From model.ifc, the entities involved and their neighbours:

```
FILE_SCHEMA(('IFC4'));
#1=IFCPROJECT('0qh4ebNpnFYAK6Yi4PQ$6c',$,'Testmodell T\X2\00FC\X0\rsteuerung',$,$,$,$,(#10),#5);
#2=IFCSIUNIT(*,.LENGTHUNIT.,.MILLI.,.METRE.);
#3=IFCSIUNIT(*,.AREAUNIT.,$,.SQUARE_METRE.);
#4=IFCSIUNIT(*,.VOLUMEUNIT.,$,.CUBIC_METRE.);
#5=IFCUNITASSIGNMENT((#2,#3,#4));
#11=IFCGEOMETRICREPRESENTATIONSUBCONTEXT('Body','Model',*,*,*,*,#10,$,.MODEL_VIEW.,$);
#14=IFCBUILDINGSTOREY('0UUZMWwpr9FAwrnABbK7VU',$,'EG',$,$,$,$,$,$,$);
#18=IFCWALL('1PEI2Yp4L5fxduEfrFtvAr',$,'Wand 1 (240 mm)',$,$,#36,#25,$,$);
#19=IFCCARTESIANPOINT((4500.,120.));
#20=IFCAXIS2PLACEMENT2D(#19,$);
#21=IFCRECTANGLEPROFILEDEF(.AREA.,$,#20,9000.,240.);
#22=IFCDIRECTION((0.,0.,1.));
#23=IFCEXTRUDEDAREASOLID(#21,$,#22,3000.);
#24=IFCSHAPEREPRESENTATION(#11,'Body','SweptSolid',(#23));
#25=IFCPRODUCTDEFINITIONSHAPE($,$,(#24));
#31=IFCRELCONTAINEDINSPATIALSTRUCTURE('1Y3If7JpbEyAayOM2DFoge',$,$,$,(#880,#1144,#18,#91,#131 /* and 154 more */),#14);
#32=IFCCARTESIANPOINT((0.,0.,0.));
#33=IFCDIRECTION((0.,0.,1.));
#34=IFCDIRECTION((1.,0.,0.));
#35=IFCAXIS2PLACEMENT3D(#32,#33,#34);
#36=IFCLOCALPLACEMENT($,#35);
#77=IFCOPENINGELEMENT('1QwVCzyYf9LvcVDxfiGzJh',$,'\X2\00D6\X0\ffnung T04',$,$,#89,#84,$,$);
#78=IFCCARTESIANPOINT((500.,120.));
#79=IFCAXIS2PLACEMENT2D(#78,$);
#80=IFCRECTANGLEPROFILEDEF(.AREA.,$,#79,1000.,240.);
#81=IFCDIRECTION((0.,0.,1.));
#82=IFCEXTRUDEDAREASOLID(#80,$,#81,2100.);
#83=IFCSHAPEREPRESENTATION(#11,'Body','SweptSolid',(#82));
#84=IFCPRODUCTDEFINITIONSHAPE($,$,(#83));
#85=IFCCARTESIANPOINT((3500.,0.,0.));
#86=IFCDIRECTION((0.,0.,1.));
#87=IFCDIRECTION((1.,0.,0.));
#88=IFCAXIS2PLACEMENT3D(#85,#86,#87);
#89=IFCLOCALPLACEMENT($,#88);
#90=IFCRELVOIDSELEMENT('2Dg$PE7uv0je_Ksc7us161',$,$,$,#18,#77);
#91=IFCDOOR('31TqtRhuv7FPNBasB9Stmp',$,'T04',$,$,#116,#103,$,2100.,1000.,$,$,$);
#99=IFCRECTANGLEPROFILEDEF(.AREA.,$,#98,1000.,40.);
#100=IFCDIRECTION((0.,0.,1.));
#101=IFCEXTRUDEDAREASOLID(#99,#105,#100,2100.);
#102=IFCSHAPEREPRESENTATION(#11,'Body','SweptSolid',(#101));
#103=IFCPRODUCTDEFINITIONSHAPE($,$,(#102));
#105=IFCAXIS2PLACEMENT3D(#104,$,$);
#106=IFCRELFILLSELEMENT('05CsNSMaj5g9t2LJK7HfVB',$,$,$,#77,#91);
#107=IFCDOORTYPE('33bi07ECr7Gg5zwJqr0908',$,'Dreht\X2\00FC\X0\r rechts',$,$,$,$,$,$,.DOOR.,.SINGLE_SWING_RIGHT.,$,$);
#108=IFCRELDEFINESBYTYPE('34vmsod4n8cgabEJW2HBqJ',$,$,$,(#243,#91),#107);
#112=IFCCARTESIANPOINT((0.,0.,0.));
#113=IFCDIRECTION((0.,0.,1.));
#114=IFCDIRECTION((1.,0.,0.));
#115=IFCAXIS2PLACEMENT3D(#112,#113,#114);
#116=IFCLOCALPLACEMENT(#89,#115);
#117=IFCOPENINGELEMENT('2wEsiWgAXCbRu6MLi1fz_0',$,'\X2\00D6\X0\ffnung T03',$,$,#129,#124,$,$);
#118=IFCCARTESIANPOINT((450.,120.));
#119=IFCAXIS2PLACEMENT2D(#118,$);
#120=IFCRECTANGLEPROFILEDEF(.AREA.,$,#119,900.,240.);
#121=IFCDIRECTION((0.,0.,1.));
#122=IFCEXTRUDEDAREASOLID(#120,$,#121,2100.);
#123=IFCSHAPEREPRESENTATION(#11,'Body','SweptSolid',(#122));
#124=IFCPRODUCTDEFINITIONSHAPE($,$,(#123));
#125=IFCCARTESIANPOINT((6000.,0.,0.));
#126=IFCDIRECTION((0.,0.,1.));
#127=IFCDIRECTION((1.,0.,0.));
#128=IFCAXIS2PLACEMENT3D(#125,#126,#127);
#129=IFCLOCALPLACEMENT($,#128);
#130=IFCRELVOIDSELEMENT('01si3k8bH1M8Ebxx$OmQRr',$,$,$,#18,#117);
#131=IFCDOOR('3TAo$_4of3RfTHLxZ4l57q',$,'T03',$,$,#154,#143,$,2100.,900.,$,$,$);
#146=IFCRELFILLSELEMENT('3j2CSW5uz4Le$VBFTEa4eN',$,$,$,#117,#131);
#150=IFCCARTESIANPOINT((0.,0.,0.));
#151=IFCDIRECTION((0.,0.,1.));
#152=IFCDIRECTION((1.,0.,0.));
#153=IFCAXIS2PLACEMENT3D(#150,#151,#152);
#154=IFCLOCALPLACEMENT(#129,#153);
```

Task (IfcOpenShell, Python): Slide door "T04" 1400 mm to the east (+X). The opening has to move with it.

```python
import ifcopenshell
import ifcopenshell.api.geometry
import ifcopenshell.util.placement

model = ifcopenshell.open("model.ifc")

door = model.by_guid("31TqtRhuv7FPNBasB9Stmp")
opening = door.FillsVoids[0].RelatingOpeningElement
wall = opening.VoidsElements[0].RelatingBuildingElement

wall_matrix = ifcopenshell.util.placement.get_local_placement(wall.ObjectPlacement)
shift = wall_matrix[:3, 0] * 1400.0
before = ifcopenshell.util.placement.get_local_placement(door.ObjectPlacement)[:3, 3].copy()

# The door is placed relative to its opening, so it follows when the opening moves.
matrix = ifcopenshell.util.placement.get_local_placement(opening.ObjectPlacement)
matrix[:3, 3] += shift
ifcopenshell.api.geometry.edit_object_placement(
    model, product=opening, matrix=matrix, is_si=False, should_transform_children=True
)

after = ifcopenshell.util.placement.get_local_placement(door.ObjectPlacement)[:3, 3]
print("door moved by", (after - before).round(3) + 0.0)

model.write("model_rev.ifc")
```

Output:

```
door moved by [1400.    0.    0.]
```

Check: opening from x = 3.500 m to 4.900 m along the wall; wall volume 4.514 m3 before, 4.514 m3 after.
